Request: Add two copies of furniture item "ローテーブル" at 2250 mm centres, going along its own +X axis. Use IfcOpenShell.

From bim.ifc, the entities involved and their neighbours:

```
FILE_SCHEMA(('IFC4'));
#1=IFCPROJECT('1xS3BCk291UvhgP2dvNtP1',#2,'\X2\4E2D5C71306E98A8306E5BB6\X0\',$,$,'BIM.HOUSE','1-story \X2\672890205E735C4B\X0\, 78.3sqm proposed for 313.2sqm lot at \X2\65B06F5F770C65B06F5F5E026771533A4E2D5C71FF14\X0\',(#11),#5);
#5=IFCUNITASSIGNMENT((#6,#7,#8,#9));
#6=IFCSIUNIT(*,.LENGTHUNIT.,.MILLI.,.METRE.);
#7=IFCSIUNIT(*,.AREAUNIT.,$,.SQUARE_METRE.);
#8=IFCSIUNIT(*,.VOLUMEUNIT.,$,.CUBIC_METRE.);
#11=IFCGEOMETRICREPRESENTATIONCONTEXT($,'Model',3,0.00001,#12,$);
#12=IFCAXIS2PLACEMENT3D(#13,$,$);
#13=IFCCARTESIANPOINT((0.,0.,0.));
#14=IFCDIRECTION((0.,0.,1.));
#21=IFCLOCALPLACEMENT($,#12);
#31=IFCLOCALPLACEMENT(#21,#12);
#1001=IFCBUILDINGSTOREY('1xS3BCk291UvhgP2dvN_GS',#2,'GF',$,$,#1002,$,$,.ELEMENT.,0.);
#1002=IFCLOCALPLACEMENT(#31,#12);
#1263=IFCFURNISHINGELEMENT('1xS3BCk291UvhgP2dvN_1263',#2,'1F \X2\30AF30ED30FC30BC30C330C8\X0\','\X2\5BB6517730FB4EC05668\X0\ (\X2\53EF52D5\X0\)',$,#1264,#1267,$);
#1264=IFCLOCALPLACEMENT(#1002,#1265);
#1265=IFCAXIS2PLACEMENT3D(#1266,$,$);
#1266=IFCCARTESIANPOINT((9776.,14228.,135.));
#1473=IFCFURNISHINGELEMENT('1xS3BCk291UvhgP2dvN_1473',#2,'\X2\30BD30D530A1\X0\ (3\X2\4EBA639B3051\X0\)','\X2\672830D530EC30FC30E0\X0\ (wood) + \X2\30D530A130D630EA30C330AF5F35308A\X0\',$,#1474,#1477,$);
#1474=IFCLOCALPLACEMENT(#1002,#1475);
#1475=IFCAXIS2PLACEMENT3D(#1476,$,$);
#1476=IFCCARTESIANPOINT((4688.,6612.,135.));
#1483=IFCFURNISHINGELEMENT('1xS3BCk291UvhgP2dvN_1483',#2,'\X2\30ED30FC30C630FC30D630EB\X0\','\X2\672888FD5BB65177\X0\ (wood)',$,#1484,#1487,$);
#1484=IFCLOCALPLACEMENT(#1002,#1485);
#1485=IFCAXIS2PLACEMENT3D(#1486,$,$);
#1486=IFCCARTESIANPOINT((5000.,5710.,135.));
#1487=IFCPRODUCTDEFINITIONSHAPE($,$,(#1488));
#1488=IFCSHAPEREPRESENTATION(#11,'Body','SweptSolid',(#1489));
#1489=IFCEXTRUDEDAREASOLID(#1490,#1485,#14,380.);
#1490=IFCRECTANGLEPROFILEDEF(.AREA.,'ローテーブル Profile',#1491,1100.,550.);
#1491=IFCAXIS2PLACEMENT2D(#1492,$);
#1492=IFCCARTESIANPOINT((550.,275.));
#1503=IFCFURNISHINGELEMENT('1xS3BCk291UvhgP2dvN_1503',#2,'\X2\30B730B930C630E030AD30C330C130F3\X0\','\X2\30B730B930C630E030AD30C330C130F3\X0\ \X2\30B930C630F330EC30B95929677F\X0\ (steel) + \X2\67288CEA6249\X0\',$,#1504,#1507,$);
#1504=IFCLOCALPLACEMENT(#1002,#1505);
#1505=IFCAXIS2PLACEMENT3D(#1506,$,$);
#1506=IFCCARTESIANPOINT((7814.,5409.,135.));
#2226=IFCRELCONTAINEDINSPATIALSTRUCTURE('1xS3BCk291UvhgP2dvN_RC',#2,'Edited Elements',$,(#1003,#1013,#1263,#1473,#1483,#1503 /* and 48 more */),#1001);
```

```python
import ifcopenshell
import ifcopenshell.api.geometry
import ifcopenshell.api.root
import ifcopenshell.util.element
import ifcopenshell.util.placement
import ifcopenshell.util.unit

model = ifcopenshell.open("bim.ifc")
unit_scale = ifcopenshell.util.unit.calculate_unit_scale(model)


def reuse_history(source, copy):
    """copy_class also copies each property set's owner history, people and application; keep the originals."""
    for rel in copy.IsDefinedBy:
        if rel.is_a("IfcRelDefinesByProperties") and (history := rel.RelatingPropertyDefinition.OwnerHistory):
            rel.RelatingPropertyDefinition.OwnerHistory = source.OwnerHistory
            ifcopenshell.util.element.remove_deep2(model, history)


source = model.by_guid("1xS3BCk291UvhgP2dvN_1483")
base = ifcopenshell.util.placement.get_local_placement(source.ObjectPlacement)
step = base[:3, 0] * 2.25 / unit_scale

for i in range(1, 3):
    copy = ifcopenshell.api.root.copy_class(model, product=source)
    copy.Representation = ifcopenshell.util.element.copy_deep(
        model, source.Representation, exclude=["IfcGeometricRepresentationContext", "IfcRepresentationMap"]
    )
    reuse_history(source, copy)
    matrix = base.copy()
    matrix[:3, 3] += i * step
    print("added at", matrix[:3, 3].round(3) + 0.0)
    ifcopenshell.api.geometry.edit_object_placement(model, product=copy, matrix=matrix, is_si=False)

model.write("bim_updated.ifc")
```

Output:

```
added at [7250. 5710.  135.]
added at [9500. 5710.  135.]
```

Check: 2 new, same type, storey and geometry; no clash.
